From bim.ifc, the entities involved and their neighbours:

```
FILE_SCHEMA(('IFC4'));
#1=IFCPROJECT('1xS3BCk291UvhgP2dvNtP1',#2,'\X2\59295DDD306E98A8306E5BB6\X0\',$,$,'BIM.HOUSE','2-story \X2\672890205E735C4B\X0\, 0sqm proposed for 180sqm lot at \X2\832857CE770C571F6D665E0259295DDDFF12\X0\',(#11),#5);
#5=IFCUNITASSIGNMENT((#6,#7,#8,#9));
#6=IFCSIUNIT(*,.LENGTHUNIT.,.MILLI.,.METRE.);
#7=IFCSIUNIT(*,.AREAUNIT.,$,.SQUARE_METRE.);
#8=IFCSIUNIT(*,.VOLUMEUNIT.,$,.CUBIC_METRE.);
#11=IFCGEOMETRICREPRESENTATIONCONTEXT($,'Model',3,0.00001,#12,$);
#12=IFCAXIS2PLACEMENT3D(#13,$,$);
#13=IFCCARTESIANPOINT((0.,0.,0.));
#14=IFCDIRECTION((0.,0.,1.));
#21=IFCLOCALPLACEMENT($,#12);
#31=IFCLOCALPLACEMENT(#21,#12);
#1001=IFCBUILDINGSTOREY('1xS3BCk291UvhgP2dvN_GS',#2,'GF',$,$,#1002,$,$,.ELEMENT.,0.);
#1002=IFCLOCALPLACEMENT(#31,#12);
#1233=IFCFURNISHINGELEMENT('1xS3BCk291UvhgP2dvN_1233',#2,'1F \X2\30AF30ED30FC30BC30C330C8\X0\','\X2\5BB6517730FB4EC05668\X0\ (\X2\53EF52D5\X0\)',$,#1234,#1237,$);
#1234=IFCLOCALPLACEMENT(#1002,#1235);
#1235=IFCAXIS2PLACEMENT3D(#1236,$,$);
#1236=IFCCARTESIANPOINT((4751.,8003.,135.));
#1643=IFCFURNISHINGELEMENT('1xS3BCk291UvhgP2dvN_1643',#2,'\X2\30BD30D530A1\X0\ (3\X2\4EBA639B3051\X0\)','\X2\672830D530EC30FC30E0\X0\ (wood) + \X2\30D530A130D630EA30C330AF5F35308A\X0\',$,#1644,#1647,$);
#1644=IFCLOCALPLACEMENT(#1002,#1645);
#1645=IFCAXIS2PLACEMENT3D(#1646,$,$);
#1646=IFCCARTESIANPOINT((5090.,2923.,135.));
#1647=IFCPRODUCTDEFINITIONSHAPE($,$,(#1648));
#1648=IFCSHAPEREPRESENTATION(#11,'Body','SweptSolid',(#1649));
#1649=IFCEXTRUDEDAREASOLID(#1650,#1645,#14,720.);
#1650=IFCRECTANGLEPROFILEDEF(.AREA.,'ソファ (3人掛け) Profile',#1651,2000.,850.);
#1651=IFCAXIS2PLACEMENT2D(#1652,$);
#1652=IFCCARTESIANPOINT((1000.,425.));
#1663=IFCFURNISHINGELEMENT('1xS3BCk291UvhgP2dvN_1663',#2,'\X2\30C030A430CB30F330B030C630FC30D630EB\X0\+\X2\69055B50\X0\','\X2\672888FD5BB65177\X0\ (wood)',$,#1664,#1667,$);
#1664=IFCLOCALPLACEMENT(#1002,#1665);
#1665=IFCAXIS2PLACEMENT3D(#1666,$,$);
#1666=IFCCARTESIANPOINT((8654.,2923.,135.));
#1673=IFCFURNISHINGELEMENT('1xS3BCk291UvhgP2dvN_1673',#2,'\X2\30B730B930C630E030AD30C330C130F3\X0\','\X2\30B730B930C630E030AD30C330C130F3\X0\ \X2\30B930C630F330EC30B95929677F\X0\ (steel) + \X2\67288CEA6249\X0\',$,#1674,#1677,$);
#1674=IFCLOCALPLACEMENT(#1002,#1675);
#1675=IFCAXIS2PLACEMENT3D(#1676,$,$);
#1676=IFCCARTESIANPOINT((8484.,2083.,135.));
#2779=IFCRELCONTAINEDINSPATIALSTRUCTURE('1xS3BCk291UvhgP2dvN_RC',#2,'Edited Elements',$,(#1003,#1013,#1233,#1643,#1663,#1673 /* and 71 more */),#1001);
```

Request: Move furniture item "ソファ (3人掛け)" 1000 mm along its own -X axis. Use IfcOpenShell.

```python
import ifcopenshell
import ifcopenshell.api.geometry
import ifcopenshell.util.placement
import ifcopenshell.util.unit

model = ifcopenshell.open("bim.ifc")
unit_scale = ifcopenshell.util.unit.calculate_unit_scale(model)

item = model.by_id(1643)
matrix = ifcopenshell.util.placement.get_local_placement(item.ObjectPlacement)
matrix[:3, 3] -= matrix[:3, 0] * 1 / unit_scale
ifcopenshell.api.geometry.edit_object_placement(model, product=item, matrix=matrix, is_si=False)

print(ifcopenshell.util.placement.get_local_placement(item.ObjectPlacement).round(3) + 0.0)

model.write("bim_edited.ifc")
```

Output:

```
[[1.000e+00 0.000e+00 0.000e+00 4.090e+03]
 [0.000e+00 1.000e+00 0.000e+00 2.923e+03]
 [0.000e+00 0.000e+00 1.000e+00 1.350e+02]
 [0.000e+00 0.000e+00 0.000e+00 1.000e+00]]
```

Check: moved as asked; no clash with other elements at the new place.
